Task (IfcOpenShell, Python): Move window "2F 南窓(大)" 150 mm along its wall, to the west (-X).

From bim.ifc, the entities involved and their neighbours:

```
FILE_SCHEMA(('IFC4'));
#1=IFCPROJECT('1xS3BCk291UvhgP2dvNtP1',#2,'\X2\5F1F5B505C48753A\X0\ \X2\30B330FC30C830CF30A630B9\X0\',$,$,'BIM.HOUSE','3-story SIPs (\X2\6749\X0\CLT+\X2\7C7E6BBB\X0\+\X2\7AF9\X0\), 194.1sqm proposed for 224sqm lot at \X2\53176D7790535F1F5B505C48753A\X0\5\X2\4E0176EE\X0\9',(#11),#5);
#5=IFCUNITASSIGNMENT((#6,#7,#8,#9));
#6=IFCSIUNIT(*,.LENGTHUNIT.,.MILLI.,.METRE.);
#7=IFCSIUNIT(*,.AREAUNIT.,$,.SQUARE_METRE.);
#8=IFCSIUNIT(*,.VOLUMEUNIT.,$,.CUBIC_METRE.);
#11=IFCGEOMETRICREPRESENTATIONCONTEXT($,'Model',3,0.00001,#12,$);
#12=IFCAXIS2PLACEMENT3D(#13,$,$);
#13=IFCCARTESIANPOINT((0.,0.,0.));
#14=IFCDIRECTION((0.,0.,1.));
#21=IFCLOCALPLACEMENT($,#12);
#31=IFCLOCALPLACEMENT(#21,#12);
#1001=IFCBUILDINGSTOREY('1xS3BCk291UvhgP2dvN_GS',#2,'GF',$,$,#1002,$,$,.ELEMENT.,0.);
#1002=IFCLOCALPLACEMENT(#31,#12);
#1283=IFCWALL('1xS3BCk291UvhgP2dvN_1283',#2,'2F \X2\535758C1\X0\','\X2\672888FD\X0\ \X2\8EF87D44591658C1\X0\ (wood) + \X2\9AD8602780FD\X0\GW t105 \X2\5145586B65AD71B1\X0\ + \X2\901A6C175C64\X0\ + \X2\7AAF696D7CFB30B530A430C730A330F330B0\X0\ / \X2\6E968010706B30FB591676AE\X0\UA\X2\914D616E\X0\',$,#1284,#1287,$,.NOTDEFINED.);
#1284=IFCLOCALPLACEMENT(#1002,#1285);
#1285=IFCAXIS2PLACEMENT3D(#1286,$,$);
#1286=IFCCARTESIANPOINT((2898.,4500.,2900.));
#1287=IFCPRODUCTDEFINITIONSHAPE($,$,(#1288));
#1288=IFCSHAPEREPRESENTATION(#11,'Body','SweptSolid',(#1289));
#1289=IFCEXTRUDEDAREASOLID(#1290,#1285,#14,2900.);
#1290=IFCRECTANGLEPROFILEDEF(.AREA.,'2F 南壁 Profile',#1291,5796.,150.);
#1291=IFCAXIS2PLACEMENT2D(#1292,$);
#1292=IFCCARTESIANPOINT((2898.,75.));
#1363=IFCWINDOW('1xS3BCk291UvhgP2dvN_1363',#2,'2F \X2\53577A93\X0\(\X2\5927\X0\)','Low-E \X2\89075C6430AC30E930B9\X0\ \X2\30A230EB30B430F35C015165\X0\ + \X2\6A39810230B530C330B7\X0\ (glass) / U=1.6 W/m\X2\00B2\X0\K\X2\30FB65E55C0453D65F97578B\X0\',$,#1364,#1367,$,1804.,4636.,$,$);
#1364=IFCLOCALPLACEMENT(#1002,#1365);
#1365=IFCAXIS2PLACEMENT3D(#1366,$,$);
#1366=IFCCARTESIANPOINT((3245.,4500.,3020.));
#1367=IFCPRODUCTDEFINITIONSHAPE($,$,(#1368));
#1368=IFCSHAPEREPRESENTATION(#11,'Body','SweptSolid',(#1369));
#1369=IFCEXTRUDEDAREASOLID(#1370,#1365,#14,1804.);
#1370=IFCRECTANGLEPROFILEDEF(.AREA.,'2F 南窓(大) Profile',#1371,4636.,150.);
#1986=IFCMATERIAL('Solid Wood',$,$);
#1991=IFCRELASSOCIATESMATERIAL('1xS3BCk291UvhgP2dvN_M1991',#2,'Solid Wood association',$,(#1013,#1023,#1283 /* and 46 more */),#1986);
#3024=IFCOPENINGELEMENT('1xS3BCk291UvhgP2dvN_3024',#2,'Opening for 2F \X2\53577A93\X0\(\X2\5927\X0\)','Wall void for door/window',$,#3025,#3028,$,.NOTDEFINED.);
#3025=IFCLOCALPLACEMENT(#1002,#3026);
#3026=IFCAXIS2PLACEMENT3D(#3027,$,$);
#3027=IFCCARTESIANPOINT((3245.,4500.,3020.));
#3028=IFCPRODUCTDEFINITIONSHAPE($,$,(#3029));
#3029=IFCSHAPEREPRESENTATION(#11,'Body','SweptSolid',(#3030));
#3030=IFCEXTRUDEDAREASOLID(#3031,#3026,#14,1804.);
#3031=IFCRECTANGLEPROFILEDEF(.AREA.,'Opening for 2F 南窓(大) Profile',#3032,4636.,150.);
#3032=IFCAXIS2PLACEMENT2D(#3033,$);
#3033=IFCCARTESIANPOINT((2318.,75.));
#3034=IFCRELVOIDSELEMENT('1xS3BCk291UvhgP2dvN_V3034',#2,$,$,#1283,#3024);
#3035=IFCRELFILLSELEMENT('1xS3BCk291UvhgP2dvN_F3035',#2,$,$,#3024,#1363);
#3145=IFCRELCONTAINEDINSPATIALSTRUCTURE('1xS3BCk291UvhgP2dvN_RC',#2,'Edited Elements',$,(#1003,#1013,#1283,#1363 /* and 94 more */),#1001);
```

```python
import ifcopenshell
import ifcopenshell.api.geometry
import ifcopenshell.util.placement

model = ifcopenshell.open("bim.ifc")

window = model.by_guid("1xS3BCk291UvhgP2dvN_1363")
opening = window.FillsVoids[0].RelatingOpeningElement
wall = opening.VoidsElements[0].RelatingBuildingElement

wall_matrix = ifcopenshell.util.placement.get_local_placement(wall.ObjectPlacement)
shift = wall_matrix[:3, 0] * -150.0
before = ifcopenshell.util.placement.get_local_placement(window.ObjectPlacement)[:3, 3].copy()

# The window is not placed relative to its opening, so move both.
for product in (opening, window):
    matrix = ifcopenshell.util.placement.get_local_placement(product.ObjectPlacement)
    matrix[:3, 3] += shift
    ifcopenshell.api.geometry.edit_object_placement(model, product=product, matrix=matrix, is_si=False)

after = ifcopenshell.util.placement.get_local_placement(window.ObjectPlacement)[:3, 3]
print("window moved by", (after - before).round(3) + 0.0)

model.write("bim_updated.ifc")
```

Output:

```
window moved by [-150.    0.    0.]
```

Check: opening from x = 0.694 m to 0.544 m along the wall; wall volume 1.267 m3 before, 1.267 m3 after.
